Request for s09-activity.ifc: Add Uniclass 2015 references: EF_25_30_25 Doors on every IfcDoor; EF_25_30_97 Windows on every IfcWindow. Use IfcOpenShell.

First a look at what the model holds.

```python
import ifcopenshell

model = ifcopenshell.open("s09-activity.ifc")
print(model.schema)
print("classifications:", [c.Name for c in model.by_type("IfcClassification")])
for ifc_class in ("IfcDoor", "IfcRoof", "IfcStair", "IfcWall", "IfcWindow"):
    print(ifc_class, len(model.by_type(ifc_class)))
```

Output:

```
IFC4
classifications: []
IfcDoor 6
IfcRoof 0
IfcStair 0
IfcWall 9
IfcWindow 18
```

```python
import ifcopenshell
import ifcopenshell.api.classification

model = ifcopenshell.open("s09-activity.ifc")

system = ifcopenshell.api.classification.add_classification(model, classification="Uniclass 2015")

codes = {
    "IfcDoor": ("EF_25_30_25", "Doors"),
    "IfcWindow": ("EF_25_30_97", "Windows"),
}
for ifc_class, (code, name) in codes.items():
    products = model.by_type(ifc_class)
    ifcopenshell.api.classification.add_reference(
        model, products=products, classification=system, identification=code, name=name
    )
    print(code, len(products))

model.write("s09-activity_edited.ifc")
```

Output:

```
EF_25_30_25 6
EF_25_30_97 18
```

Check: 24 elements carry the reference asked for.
